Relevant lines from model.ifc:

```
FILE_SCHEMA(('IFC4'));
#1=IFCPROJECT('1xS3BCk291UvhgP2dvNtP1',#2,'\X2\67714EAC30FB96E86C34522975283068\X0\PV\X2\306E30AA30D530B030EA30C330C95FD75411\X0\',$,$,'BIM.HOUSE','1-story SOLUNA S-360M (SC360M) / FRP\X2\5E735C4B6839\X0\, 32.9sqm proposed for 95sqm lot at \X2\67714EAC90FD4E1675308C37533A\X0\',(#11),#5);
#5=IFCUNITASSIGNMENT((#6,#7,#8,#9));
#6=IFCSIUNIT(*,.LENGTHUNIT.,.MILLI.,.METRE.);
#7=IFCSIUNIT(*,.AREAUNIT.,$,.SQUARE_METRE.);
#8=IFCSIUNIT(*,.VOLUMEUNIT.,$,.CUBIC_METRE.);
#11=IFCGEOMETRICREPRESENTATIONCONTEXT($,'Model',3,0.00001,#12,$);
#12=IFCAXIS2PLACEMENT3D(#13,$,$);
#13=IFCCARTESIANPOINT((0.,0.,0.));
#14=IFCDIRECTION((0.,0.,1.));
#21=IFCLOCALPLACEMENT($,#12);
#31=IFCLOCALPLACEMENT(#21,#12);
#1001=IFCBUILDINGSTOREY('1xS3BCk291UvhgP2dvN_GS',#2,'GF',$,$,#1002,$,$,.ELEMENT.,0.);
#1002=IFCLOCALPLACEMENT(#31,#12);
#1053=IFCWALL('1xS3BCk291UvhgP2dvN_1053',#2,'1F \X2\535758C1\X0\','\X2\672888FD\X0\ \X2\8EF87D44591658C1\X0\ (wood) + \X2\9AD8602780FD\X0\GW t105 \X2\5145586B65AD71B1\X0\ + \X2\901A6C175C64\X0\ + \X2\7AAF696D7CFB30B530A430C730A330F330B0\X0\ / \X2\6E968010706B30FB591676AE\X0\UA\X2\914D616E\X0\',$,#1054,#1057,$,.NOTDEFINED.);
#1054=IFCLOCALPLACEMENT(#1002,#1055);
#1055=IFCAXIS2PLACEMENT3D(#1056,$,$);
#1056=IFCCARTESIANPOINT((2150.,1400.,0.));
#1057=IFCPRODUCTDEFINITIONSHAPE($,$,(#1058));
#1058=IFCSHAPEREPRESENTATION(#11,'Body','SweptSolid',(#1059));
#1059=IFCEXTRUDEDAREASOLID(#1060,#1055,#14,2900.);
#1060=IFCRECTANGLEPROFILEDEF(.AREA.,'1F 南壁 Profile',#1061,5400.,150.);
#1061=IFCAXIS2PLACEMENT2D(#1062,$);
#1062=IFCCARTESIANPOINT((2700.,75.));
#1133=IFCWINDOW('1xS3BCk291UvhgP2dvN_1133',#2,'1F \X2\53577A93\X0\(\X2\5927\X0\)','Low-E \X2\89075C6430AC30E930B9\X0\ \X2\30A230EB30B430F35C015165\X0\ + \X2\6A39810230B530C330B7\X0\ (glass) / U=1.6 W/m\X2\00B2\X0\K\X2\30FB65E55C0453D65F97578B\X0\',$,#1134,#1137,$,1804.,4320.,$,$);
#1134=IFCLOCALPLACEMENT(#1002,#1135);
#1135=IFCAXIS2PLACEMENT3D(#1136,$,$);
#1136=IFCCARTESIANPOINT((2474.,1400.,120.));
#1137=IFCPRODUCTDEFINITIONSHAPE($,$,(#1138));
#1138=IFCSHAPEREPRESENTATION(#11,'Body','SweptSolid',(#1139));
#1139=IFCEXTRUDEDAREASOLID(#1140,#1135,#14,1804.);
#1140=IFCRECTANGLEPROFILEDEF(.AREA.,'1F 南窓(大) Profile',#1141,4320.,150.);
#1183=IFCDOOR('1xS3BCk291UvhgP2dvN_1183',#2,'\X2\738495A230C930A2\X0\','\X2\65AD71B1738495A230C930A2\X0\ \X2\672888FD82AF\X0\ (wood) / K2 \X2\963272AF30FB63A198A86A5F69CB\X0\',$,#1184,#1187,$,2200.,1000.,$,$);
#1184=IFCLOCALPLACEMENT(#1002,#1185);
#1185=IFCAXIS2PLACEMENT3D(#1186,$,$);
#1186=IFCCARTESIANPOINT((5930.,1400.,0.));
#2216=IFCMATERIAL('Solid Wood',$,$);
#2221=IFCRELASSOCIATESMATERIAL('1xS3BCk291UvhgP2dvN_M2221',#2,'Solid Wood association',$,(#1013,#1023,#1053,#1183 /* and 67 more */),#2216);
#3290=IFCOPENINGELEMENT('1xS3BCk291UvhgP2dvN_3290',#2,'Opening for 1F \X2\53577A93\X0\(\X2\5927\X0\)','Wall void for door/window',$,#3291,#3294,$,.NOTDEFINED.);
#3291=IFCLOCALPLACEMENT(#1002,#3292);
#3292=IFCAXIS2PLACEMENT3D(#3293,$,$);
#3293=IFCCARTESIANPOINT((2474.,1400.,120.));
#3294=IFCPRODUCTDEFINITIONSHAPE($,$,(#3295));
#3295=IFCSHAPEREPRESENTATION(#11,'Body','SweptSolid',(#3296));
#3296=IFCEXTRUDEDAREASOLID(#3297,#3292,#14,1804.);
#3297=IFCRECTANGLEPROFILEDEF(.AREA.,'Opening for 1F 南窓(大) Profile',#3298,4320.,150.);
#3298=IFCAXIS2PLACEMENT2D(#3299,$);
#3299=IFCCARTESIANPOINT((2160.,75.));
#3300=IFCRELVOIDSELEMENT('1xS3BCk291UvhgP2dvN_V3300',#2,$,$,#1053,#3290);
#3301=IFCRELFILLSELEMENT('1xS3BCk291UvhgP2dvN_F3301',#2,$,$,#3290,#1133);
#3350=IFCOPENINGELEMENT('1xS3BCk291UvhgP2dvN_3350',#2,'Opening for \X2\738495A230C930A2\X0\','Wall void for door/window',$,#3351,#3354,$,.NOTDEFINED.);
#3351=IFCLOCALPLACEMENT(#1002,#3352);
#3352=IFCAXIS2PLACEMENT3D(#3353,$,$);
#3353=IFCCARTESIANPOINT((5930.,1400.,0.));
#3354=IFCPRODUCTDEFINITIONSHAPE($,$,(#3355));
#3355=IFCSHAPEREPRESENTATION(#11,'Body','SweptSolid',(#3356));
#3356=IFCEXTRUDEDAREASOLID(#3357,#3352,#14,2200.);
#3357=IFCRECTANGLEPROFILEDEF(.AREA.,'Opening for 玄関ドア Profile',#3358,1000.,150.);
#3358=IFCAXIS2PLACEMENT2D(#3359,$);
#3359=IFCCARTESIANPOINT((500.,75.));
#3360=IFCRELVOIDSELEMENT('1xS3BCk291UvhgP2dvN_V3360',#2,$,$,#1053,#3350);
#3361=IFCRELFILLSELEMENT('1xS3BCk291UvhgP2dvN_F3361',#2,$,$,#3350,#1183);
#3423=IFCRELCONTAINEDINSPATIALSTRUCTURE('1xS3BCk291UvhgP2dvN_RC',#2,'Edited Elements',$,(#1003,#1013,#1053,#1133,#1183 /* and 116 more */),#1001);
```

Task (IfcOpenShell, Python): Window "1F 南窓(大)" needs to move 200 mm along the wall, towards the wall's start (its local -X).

```python
import ifcopenshell
import ifcopenshell.api.geometry
import ifcopenshell.util.placement

model = ifcopenshell.open("model.ifc")

window = model.by_guid("1xS3BCk291UvhgP2dvN_1133")
opening = window.FillsVoids[0].RelatingOpeningElement
wall = opening.VoidsElements[0].RelatingBuildingElement

wall_matrix = ifcopenshell.util.placement.get_local_placement(wall.ObjectPlacement)
shift = wall_matrix[:3, 0] * -200.0
before = ifcopenshell.util.placement.get_local_placement(window.ObjectPlacement)[:3, 3].copy()

# The window is not placed relative to its opening, so move both.
for product in (opening, window):
    matrix = ifcopenshell.util.placement.get_local_placement(product.ObjectPlacement)
    matrix[:3, 3] += shift
    ifcopenshell.api.geometry.edit_object_placement(model, product=product, matrix=matrix, is_si=False)

after = ifcopenshell.util.placement.get_local_placement(window.ObjectPlacement)[:3, 3]
print("window moved by", (after - before).round(3) + 0.0)

model.write("model_rev.ifc")
```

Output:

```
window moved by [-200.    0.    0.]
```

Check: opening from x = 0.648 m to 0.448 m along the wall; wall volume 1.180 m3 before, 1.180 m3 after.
